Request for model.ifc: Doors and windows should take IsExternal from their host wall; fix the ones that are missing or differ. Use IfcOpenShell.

First a look at what the model holds.

```python
import ifcopenshell
import ifcopenshell.util.element

model = ifcopenshell.open("model.ifc")
print(model.schema)
seen = {}
for e in model.by_type("IfcDoor") + model.by_type("IfcWindow"):
    if not e.FillsVoids:
        continue
    host = e.FillsVoids[0].RelatingOpeningElement.VoidsElements[0].RelatingBuildingElement
    own = ifcopenshell.util.element.get_pset(e, f"Pset_{e.is_a()[3:].removesuffix('StandardCase')}Common", "IsExternal")
    wall = ifcopenshell.util.element.get_pset(host, "Pset_WallCommon", "IsExternal")
    seen[e.is_a(), own, wall] = seen.get((e.is_a(), own, wall), 0) + 1
for (cls, own, wall), count in sorted(seen.items(), key=str):
    print(count, cls, "IsExternal:", own, "| host wall:", wall)
```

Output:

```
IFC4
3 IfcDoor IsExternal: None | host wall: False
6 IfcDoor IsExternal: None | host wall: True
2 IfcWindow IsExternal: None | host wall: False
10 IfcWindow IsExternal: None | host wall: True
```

```python
import ifcopenshell
import ifcopenshell.api.pset
import ifcopenshell.util.element

model = ifcopenshell.open("model.ifc")

count = 0
for ifc_class, pset_name in (("IfcDoor", "Pset_DoorCommon"), ("IfcWindow", "Pset_WindowCommon")):
    for e in model.by_type(ifc_class):
        if not e.FillsVoids:
            continue
        host = e.FillsVoids[0].RelatingOpeningElement.VoidsElements[0].RelatingBuildingElement
        external = ifcopenshell.util.element.get_pset(host, "Pset_WallCommon", "IsExternal")
        if external is None or ifcopenshell.util.element.get_pset(e, pset_name, "IsExternal") == external:
            continue
        pset = ifcopenshell.api.pset.add_pset(model, product=e, name=pset_name)
        ifcopenshell.api.pset.edit_pset(model, pset=pset, properties={"IsExternal": external})
        count += 1

print(count, "updated")

model.write("model-out.ifc")
```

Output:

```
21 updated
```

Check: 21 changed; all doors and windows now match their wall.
